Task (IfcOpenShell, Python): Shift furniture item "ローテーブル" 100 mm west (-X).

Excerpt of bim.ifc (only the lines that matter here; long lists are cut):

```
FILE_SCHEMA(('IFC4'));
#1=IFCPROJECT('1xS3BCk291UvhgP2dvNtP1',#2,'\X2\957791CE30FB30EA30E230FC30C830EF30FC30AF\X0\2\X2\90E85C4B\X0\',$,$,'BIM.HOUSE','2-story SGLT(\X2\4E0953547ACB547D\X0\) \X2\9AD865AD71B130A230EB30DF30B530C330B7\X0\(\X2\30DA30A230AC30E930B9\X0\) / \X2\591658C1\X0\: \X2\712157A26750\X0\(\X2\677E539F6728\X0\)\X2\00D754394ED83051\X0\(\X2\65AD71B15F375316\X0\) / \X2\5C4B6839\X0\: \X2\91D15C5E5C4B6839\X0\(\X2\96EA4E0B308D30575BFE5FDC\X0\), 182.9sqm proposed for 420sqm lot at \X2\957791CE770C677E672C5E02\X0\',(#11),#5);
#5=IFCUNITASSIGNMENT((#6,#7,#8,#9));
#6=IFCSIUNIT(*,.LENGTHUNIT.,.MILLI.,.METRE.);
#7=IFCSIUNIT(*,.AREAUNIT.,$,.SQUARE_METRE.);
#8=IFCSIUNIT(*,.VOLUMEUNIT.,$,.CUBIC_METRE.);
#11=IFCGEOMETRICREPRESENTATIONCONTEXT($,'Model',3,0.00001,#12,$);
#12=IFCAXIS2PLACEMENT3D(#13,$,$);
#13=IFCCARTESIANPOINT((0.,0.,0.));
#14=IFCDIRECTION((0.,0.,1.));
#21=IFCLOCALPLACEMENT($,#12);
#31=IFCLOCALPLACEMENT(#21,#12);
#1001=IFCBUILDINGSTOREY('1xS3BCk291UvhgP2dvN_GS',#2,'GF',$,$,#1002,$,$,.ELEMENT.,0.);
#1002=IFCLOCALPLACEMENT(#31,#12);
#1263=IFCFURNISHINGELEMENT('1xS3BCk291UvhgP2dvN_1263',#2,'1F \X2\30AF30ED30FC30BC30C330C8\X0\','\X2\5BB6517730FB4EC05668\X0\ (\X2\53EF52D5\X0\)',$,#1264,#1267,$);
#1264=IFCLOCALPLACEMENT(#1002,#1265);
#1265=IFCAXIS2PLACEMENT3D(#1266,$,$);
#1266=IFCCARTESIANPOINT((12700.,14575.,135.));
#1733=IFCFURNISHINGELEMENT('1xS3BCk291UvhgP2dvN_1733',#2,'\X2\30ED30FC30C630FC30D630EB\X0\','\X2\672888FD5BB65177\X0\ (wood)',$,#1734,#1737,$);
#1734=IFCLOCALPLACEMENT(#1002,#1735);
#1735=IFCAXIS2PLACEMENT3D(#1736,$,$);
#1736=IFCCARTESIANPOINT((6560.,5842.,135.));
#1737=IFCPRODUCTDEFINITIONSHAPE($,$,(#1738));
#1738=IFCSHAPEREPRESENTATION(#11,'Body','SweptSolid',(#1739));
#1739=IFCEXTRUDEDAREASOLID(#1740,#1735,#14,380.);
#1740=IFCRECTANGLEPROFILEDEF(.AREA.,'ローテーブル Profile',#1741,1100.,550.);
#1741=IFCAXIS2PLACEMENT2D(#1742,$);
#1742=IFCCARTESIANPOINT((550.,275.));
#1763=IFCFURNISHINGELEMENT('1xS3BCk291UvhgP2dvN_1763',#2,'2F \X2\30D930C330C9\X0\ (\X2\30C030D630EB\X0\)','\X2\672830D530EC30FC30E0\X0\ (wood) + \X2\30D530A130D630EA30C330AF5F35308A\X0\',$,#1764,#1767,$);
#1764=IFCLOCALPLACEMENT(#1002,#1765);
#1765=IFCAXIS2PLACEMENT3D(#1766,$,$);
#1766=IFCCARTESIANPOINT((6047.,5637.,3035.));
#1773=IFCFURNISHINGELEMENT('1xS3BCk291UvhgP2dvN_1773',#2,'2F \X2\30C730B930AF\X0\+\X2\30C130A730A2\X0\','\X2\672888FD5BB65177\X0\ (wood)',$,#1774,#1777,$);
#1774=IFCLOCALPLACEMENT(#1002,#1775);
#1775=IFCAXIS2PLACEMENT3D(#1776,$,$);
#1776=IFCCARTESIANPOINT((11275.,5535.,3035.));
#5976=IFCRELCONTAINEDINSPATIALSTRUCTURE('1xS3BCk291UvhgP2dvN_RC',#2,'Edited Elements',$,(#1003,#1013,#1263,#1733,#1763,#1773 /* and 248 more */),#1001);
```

```python
import ifcopenshell
import ifcopenshell.api.geometry
import ifcopenshell.util.placement
import ifcopenshell.util.unit

model = ifcopenshell.open("bim.ifc")
unit_scale = ifcopenshell.util.unit.calculate_unit_scale(model)

item = model.by_id(1733)
matrix = ifcopenshell.util.placement.get_local_placement(item.ObjectPlacement)
matrix[0, 3] -= 0.1 / unit_scale
ifcopenshell.api.geometry.edit_object_placement(model, product=item, matrix=matrix, is_si=False)

print(ifcopenshell.util.placement.get_local_placement(item.ObjectPlacement).round(3) + 0.0)

model.write("bim-out.ifc")
```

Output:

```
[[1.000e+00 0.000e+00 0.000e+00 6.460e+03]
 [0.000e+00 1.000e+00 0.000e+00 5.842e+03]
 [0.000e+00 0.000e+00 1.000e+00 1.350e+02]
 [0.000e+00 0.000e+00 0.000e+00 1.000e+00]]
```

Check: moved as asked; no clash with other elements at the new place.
